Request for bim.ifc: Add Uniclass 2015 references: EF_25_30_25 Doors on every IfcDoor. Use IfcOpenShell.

First a look at what the model holds.

```python
import ifcopenshell

model = ifcopenshell.open("bim.ifc")
print(model.schema)
print("classifications:", [c.Name for c in model.by_type("IfcClassification")])
for ifc_class in ("IfcDoor", "IfcRoof", "IfcStair", "IfcWall", "IfcWindow"):
    print(ifc_class, len(model.by_type(ifc_class)))
```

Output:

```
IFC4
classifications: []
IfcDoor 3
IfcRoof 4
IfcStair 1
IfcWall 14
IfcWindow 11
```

```python
import ifcopenshell
import ifcopenshell.api.classification

model = ifcopenshell.open("bim.ifc")

system = ifcopenshell.api.classification.add_classification(model, classification="Uniclass 2015")

codes = {
    "IfcDoor": ("EF_25_30_25", "Doors"),
}
for ifc_class, (code, name) in codes.items():
    products = model.by_type(ifc_class)
    ifcopenshell.api.classification.add_reference(
        model, products=products, classification=system, identification=code, name=name
    )
    print(code, len(products))

model.write("bim_updated.ifc")
```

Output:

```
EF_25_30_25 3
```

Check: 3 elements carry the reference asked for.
